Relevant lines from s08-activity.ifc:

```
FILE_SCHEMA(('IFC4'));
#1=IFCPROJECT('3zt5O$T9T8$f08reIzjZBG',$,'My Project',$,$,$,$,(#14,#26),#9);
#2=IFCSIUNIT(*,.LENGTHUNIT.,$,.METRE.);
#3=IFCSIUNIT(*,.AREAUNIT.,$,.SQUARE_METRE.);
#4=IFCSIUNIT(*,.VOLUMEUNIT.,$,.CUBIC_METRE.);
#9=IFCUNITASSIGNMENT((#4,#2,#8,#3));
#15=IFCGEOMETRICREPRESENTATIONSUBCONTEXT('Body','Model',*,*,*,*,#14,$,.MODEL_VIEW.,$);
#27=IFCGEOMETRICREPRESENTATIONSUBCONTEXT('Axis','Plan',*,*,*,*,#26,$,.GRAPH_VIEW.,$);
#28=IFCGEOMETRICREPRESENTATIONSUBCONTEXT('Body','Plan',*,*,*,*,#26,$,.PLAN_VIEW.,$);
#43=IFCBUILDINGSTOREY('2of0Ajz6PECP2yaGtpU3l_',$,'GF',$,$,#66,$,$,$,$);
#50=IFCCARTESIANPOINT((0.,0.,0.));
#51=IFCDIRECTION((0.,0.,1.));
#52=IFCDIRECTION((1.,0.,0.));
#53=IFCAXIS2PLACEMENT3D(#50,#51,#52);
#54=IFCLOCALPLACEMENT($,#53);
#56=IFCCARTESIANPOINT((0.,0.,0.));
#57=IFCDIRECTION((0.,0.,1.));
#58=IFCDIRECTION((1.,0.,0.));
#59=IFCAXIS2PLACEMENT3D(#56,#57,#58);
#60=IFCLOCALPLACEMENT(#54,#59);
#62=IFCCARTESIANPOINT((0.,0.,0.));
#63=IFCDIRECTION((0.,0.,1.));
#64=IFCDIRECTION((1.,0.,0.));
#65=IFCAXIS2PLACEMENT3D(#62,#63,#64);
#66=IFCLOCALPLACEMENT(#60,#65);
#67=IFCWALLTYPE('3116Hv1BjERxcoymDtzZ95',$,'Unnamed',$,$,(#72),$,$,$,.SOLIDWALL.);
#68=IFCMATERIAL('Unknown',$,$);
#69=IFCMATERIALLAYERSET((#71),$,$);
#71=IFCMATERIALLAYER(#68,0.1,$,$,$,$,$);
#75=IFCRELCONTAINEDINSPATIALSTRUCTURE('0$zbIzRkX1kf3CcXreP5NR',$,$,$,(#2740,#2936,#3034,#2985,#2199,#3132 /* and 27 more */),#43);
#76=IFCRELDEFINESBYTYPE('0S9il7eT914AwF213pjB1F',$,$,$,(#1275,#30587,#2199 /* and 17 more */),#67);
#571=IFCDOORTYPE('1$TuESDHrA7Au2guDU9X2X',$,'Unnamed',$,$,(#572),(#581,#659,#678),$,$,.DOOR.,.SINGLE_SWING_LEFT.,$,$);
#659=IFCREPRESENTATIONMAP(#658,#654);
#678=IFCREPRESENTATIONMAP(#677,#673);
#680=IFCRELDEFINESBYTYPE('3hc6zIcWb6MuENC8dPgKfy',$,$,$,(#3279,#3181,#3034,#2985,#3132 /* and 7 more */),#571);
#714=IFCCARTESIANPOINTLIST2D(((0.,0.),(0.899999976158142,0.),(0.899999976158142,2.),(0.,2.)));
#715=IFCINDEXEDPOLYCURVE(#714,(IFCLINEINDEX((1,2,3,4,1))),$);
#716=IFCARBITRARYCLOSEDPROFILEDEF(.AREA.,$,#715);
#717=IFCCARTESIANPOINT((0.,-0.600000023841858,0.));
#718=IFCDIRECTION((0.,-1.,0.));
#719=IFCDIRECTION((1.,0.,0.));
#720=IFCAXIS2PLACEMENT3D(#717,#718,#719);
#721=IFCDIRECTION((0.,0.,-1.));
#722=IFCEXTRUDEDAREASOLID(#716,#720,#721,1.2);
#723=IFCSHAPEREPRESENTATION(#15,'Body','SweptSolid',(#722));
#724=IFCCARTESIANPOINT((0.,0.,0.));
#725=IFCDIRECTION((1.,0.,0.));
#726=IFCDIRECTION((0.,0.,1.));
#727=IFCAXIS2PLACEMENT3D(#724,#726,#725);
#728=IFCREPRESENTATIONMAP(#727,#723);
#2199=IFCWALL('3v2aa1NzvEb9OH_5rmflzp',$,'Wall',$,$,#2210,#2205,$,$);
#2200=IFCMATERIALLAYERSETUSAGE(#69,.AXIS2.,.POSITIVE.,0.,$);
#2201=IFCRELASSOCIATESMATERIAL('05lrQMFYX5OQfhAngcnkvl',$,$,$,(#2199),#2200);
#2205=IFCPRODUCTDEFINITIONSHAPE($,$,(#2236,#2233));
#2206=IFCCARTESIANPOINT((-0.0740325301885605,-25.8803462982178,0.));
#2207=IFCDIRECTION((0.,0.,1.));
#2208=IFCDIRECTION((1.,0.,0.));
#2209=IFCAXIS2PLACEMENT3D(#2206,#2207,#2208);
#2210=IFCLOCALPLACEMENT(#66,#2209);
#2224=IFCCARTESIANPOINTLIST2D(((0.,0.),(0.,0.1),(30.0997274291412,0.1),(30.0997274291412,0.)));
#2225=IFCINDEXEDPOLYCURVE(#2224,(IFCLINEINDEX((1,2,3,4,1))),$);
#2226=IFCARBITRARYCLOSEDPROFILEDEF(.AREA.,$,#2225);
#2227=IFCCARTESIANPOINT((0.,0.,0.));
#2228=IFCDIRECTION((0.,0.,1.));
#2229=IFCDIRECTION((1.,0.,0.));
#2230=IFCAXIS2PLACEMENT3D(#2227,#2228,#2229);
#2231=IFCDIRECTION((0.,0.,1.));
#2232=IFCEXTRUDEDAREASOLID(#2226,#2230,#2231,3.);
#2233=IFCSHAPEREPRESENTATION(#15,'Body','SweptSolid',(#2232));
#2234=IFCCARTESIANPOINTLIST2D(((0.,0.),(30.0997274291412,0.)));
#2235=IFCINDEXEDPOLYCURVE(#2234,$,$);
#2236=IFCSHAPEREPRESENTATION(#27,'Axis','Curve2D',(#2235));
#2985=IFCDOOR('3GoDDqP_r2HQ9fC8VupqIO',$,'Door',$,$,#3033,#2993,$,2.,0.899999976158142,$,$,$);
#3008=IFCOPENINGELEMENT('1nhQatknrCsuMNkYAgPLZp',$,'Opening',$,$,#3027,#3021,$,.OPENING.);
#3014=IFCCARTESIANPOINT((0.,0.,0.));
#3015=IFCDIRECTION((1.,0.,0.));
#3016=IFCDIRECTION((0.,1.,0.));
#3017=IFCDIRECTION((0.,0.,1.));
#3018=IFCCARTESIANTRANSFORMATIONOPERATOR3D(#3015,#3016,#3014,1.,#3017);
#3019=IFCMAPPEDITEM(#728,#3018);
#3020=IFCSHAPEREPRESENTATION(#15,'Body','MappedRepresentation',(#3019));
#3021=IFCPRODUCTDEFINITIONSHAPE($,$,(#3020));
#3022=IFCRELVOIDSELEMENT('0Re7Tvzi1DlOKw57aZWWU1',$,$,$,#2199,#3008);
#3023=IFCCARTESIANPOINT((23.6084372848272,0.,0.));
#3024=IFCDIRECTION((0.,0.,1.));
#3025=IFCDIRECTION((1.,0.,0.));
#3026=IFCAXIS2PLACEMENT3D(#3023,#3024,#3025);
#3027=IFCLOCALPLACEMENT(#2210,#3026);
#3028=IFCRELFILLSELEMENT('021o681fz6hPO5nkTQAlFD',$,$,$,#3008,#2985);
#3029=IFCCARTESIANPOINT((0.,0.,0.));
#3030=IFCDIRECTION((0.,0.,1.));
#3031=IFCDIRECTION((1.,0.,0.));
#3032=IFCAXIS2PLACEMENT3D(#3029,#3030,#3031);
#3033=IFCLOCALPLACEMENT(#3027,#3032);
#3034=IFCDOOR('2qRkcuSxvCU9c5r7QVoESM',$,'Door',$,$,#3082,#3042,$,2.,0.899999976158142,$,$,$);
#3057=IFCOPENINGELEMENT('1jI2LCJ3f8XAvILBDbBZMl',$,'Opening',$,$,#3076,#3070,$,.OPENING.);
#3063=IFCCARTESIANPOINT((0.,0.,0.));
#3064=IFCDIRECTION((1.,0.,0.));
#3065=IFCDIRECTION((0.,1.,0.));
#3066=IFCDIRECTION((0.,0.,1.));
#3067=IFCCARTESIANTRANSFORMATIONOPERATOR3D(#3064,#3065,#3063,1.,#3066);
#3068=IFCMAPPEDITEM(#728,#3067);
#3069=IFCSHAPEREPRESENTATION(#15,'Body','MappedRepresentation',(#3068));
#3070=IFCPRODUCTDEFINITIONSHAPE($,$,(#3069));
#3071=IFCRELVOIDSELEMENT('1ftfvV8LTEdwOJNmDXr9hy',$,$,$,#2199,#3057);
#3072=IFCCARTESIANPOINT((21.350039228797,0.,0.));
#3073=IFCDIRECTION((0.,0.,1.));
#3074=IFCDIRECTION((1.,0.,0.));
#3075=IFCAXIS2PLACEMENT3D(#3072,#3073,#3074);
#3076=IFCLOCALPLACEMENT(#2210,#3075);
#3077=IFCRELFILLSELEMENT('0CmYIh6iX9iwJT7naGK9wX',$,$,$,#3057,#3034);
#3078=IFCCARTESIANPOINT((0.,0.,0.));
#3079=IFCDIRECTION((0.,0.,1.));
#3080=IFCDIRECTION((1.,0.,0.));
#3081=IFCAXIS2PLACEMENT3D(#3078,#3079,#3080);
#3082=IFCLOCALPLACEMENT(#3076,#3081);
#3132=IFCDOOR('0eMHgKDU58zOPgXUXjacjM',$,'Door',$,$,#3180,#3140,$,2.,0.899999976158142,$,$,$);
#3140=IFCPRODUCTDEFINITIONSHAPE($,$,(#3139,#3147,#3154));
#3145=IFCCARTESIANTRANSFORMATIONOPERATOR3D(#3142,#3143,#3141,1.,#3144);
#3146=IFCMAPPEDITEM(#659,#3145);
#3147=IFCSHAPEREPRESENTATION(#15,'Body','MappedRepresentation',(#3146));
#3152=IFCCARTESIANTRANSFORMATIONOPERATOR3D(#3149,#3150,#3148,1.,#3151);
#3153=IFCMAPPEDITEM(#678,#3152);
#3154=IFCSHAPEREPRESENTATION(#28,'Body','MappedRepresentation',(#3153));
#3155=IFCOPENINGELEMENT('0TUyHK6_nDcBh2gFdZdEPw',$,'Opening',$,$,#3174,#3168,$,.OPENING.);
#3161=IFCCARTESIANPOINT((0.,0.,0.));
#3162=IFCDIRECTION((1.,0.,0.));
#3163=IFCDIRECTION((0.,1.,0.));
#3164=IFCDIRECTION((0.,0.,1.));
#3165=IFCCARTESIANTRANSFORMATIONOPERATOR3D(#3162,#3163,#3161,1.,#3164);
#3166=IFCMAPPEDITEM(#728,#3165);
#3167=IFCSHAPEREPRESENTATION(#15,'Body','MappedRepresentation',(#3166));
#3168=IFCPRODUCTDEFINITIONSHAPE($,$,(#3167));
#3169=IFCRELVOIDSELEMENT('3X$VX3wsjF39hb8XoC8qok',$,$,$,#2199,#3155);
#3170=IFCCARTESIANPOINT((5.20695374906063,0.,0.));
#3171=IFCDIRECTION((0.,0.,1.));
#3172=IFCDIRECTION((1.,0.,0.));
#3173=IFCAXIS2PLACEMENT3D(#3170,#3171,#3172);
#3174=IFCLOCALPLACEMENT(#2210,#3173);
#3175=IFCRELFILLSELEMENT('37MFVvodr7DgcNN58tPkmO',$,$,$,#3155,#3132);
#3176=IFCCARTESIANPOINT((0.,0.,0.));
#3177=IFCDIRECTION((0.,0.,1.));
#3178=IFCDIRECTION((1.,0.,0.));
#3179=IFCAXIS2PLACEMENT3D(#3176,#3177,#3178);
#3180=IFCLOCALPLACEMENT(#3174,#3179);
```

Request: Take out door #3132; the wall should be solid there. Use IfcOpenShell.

```python
import ifcopenshell
import ifcopenshell.api.feature
import ifcopenshell.api.root
import ifcopenshell.geom
import ifcopenshell.util.shape

model = ifcopenshell.open("s08-activity.ifc")
settings = ifcopenshell.geom.settings()


def volume(element):
    """Net volume in cubic metres, openings subtracted."""
    shape = ifcopenshell.geom.create_shape(settings, element)
    return ifcopenshell.util.shape.get_volume(shape.geometry)


door = model.by_guid("0eMHgKDU58zOPgXUXjacjM")
opening = door.FillsVoids[0].RelatingOpeningElement
wall = opening.VoidsElements[0].RelatingBuildingElement
before = volume(wall)

ifcopenshell.api.root.remove_product(model, product=door)
ifcopenshell.api.feature.remove_feature(model, feature=opening)

after = volume(wall)

print(f"wall volume {before:.3f} -> {after:.3f} m3")

model.write("s08-activity-out.ifc")
```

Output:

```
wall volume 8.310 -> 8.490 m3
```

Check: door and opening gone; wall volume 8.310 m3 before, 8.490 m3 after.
